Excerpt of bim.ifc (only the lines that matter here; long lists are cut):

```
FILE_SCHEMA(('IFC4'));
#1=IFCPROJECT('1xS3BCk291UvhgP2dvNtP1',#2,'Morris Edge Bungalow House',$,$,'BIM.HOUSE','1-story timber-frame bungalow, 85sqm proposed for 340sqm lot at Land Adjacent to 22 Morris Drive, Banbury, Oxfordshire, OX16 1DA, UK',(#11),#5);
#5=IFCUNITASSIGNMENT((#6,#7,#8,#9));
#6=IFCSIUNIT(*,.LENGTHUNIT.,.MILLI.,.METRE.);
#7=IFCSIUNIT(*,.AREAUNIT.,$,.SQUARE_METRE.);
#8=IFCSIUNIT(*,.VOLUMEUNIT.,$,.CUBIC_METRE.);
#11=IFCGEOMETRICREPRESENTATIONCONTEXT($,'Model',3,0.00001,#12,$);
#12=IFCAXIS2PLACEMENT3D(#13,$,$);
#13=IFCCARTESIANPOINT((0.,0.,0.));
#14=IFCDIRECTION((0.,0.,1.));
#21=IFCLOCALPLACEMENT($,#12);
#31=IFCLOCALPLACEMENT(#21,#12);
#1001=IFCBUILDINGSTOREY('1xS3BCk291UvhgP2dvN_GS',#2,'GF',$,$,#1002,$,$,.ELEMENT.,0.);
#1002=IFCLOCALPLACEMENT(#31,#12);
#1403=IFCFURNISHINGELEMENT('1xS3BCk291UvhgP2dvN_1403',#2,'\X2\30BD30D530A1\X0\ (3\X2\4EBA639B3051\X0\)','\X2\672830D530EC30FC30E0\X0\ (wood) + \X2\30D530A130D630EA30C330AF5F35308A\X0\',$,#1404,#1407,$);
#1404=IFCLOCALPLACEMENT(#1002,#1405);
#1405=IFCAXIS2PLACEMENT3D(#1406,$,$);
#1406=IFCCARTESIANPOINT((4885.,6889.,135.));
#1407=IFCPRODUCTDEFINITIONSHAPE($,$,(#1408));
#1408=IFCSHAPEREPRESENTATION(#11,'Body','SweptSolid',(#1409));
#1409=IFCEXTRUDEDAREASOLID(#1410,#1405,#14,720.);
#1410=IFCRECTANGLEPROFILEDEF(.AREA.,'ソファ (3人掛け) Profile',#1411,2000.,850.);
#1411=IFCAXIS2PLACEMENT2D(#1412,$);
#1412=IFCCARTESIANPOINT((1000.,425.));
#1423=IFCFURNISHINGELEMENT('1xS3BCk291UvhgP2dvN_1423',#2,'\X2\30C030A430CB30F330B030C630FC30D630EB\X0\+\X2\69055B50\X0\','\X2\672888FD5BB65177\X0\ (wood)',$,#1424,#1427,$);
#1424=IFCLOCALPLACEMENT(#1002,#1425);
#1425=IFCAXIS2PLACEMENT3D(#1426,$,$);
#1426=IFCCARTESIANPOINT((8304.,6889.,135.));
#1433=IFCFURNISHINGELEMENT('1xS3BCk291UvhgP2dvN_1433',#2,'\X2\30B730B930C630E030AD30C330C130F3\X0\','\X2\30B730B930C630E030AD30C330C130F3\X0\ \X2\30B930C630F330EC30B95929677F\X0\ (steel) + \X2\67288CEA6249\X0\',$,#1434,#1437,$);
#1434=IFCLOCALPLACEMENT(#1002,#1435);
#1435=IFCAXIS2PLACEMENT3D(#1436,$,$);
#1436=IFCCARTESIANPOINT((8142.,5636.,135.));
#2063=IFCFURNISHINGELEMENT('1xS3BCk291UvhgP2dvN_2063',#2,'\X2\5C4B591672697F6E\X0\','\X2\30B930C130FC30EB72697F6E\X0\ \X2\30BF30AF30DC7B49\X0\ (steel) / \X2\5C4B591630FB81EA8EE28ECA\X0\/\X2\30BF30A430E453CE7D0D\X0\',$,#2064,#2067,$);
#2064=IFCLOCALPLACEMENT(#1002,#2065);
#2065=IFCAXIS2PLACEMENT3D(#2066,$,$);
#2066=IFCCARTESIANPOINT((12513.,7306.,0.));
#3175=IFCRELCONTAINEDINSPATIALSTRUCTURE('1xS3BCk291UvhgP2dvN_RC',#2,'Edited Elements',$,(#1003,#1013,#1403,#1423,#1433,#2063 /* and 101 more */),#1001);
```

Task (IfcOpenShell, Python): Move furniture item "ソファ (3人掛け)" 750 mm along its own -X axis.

```python
import ifcopenshell
import ifcopenshell.api.geometry
import ifcopenshell.util.placement

model = ifcopenshell.open("bim.ifc")

item = model.by_id(1403)
matrix = ifcopenshell.util.placement.get_local_placement(item.ObjectPlacement)
matrix[:3, 3] -= matrix[:3, 0] * 750.0
ifcopenshell.api.geometry.edit_object_placement(model, product=item, matrix=matrix, is_si=False)

print(ifcopenshell.util.placement.get_local_placement(item.ObjectPlacement).round(3) + 0.0)

model.write("bim-out.ifc")
```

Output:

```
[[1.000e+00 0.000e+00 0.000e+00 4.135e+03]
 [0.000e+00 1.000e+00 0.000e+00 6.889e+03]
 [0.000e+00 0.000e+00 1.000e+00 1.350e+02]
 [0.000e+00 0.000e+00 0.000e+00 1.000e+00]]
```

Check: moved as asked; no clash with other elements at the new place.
